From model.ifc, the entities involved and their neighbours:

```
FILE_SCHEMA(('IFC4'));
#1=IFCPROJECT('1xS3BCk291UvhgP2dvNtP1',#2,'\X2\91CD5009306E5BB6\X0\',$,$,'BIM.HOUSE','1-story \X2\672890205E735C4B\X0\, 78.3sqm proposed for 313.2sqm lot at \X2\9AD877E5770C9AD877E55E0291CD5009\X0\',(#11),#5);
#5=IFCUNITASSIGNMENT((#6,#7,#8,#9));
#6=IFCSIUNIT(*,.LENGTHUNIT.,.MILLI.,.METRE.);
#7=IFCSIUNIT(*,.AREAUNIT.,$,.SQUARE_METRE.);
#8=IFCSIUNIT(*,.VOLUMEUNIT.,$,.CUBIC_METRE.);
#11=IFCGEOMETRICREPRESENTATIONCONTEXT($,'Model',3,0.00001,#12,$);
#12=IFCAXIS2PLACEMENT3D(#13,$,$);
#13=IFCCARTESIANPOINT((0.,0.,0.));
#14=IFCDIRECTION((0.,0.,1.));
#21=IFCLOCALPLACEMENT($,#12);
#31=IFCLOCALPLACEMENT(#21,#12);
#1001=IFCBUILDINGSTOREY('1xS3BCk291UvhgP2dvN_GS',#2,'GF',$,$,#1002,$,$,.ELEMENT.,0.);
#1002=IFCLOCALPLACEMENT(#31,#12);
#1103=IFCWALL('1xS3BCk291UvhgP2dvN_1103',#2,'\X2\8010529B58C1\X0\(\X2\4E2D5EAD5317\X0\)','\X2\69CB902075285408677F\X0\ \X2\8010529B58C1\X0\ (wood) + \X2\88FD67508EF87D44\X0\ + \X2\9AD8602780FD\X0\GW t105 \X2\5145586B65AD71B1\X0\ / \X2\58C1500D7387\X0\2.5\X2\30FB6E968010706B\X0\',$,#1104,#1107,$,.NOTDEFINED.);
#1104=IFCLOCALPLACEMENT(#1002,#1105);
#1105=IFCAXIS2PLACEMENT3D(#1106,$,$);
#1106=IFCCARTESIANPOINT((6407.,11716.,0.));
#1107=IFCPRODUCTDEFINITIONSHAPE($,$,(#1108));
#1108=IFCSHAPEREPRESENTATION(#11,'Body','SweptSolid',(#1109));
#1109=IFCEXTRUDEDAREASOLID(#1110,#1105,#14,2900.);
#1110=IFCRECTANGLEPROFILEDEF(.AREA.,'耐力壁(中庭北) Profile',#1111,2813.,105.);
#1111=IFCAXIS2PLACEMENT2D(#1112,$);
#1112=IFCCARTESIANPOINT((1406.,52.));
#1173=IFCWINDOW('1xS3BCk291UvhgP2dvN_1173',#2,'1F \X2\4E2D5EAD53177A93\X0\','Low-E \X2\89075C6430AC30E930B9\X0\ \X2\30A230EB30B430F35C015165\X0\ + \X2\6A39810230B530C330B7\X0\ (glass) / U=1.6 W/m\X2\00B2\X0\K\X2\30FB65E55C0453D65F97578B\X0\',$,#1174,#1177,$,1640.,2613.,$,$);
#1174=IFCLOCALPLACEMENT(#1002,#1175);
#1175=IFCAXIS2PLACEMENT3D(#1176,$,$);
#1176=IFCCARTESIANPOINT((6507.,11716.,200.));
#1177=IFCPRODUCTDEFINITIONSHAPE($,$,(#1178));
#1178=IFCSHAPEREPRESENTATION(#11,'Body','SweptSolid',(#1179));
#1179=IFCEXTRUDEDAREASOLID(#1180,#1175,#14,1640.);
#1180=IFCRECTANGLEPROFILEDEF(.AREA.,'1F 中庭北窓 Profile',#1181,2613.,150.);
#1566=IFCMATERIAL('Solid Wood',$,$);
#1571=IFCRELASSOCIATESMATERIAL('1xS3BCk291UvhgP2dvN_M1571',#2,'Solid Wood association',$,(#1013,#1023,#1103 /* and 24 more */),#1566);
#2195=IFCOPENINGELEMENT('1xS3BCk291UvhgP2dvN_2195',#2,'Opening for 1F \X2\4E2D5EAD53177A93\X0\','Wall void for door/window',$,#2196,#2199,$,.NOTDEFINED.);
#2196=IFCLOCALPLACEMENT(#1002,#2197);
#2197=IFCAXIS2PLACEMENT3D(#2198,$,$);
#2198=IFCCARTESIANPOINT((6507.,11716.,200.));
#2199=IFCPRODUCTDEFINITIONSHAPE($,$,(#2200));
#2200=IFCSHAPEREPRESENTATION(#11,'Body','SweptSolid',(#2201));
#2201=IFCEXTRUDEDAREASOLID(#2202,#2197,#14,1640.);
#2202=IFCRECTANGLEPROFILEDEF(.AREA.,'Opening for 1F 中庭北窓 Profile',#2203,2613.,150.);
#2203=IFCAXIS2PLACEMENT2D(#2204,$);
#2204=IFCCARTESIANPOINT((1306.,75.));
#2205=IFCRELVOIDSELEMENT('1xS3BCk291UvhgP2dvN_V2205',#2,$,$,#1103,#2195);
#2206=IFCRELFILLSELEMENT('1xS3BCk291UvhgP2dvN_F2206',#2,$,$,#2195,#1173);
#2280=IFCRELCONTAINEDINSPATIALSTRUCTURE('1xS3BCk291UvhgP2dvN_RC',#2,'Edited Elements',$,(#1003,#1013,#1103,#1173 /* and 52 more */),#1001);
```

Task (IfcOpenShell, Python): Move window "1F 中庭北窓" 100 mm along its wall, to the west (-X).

```python
import ifcopenshell
import ifcopenshell.api.geometry
import ifcopenshell.util.placement

model = ifcopenshell.open("model.ifc")

window = model.by_guid("1xS3BCk291UvhgP2dvN_1173")
opening = window.FillsVoids[0].RelatingOpeningElement
wall = opening.VoidsElements[0].RelatingBuildingElement

wall_matrix = ifcopenshell.util.placement.get_local_placement(wall.ObjectPlacement)
shift = wall_matrix[:3, 0] * -100.0
before = ifcopenshell.util.placement.get_local_placement(window.ObjectPlacement)[:3, 3].copy()

# The window is not placed relative to its opening, so move both.
for product in (opening, window):
    matrix = ifcopenshell.util.placement.get_local_placement(product.ObjectPlacement)
    matrix[:3, 3] += shift
    ifcopenshell.api.geometry.edit_object_placement(model, product=product, matrix=matrix, is_si=False)

after = ifcopenshell.util.placement.get_local_placement(window.ObjectPlacement)[:3, 3]
print("window moved by", (after - before).round(3) + 0.0)

model.write("model_updated.ifc")
```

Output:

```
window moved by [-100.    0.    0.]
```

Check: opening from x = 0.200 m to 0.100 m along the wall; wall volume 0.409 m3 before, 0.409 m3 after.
